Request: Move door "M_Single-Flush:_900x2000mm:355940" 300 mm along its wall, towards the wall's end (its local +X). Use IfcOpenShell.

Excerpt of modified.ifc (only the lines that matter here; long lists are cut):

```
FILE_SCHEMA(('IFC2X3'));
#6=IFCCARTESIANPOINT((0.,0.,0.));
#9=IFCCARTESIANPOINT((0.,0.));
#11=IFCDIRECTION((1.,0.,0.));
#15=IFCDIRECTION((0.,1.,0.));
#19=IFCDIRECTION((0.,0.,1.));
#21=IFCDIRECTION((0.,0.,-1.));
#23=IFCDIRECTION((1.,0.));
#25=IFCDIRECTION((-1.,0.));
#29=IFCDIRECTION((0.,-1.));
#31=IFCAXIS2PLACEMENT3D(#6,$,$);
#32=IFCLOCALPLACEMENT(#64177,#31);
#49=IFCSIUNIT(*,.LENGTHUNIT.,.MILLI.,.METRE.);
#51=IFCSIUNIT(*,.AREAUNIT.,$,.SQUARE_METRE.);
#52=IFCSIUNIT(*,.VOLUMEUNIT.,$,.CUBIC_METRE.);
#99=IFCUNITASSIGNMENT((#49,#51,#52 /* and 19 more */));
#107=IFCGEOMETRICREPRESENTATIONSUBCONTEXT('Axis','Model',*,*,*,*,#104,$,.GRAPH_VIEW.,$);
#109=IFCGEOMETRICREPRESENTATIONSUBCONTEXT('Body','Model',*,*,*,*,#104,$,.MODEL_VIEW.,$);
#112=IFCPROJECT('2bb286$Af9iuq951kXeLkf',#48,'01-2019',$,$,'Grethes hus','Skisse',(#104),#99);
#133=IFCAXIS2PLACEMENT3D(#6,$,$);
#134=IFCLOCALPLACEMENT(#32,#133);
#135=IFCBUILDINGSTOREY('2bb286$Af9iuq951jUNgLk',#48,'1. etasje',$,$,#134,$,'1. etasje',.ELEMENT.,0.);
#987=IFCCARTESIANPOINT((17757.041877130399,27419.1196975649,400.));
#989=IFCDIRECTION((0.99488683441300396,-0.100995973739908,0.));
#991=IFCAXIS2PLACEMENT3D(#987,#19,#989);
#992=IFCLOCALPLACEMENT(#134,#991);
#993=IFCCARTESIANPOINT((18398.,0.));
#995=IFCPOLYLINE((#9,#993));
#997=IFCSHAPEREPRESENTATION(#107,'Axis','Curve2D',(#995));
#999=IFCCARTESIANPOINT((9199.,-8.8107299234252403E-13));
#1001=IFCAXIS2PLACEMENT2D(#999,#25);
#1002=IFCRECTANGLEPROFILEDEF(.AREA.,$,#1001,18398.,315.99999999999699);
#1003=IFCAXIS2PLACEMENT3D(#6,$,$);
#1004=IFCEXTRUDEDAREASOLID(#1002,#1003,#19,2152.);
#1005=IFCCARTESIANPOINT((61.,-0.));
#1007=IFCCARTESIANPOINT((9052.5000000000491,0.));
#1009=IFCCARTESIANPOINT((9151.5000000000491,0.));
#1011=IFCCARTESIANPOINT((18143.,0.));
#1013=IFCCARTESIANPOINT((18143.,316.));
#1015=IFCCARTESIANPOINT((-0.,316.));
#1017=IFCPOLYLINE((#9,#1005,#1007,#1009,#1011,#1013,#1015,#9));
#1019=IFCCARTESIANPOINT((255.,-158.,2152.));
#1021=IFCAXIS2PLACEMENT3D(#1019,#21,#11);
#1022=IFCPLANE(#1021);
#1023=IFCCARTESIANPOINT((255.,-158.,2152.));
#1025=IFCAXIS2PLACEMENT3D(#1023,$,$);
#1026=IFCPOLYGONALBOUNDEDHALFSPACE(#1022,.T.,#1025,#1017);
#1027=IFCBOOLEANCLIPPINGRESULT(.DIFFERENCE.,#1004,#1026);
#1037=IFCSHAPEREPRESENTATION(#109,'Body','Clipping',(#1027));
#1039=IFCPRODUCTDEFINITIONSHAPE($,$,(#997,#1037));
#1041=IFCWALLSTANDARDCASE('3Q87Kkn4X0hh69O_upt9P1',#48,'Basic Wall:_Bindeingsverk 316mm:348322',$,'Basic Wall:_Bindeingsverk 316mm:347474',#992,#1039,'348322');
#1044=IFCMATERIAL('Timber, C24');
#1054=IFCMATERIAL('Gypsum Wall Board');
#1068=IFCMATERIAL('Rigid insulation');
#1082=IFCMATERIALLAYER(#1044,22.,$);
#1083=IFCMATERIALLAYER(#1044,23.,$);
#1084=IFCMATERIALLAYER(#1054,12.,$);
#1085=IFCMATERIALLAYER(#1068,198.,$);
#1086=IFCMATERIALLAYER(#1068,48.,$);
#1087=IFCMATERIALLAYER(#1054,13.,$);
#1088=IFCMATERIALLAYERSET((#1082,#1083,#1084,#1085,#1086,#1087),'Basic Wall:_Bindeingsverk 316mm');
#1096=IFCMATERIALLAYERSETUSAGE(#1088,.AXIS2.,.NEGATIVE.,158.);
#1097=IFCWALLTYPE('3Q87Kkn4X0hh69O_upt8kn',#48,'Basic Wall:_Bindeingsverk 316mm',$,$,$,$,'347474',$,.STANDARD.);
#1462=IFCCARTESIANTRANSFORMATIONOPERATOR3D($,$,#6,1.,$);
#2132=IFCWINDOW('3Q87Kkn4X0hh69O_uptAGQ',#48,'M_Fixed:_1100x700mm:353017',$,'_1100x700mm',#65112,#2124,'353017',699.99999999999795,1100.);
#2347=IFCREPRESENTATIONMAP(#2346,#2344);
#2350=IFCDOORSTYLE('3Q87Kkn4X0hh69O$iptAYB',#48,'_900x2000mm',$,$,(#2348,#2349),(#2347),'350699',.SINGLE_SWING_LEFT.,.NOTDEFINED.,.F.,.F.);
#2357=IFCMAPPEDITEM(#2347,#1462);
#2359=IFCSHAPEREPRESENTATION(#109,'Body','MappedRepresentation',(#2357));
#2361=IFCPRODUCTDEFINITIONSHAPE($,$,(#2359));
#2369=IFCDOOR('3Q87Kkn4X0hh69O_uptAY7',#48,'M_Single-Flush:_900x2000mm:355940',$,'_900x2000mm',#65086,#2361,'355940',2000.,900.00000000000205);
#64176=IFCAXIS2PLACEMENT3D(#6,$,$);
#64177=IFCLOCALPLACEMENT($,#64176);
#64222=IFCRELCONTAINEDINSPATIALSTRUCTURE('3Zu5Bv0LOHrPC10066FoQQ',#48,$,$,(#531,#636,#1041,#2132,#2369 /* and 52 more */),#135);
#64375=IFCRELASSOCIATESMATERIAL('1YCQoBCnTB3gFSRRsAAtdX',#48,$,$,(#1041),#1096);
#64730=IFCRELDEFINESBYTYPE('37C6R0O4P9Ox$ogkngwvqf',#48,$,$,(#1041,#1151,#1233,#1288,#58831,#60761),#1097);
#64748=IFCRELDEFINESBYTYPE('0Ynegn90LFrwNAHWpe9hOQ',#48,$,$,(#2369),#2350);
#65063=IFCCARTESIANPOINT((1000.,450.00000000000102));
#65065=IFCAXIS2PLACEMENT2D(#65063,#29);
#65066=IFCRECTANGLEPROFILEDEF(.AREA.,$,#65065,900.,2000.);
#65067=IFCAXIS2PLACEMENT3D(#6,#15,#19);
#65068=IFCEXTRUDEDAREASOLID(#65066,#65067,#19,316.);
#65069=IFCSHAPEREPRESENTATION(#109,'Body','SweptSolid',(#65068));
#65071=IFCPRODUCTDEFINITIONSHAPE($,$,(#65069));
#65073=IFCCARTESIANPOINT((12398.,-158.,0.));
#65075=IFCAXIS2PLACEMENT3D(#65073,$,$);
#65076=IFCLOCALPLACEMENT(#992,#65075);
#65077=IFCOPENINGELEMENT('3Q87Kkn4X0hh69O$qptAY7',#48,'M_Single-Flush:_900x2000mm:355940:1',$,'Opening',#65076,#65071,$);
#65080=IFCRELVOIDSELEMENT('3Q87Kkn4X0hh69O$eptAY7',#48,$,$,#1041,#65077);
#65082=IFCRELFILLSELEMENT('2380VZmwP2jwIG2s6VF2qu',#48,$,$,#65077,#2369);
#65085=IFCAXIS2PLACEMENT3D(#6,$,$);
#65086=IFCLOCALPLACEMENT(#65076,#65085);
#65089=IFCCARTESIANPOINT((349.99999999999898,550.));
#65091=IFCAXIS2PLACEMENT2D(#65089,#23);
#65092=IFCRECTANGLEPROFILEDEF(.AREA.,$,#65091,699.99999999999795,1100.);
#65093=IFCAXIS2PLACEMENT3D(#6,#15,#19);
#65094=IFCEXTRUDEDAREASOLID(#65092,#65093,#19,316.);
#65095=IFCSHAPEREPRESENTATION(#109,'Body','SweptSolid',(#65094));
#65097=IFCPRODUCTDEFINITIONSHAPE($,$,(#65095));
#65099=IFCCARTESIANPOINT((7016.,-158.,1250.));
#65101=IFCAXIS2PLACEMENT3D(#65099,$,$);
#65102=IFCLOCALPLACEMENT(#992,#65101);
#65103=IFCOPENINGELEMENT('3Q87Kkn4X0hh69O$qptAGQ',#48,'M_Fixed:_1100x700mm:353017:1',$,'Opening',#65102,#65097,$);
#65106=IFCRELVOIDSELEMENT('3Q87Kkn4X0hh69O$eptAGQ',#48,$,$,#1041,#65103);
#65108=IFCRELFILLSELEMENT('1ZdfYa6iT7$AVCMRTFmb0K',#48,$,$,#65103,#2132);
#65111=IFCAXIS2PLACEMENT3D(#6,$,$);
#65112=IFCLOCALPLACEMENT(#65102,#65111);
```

```python
import ifcopenshell
import ifcopenshell.api.geometry
import ifcopenshell.util.placement
import ifcopenshell.util.unit

model = ifcopenshell.open("modified.ifc")
unit_scale = ifcopenshell.util.unit.calculate_unit_scale(model)

door = model.by_guid("3Q87Kkn4X0hh69O_uptAY7")
opening = door.FillsVoids[0].RelatingOpeningElement
wall = opening.VoidsElements[0].RelatingBuildingElement

wall_matrix = ifcopenshell.util.placement.get_local_placement(wall.ObjectPlacement)
shift = wall_matrix[:3, 0] * 0.3 / unit_scale
before = ifcopenshell.util.placement.get_local_placement(door.ObjectPlacement)[:3, 3].copy()

# The door is placed relative to its opening, so it follows when the opening moves.
matrix = ifcopenshell.util.placement.get_local_placement(opening.ObjectPlacement)
matrix[:3, 3] += shift
ifcopenshell.api.geometry.edit_object_placement(
    model, product=opening, matrix=matrix, is_si=False, should_transform_children=True
)

after = ifcopenshell.util.placement.get_local_placement(door.ObjectPlacement)[:3, 3]
print("door moved by", (after - before).round(3) + 0.0)

model.write("modified-out.ifc")
```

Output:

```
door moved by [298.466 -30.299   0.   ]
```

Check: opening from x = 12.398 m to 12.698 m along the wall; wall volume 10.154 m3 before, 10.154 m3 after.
